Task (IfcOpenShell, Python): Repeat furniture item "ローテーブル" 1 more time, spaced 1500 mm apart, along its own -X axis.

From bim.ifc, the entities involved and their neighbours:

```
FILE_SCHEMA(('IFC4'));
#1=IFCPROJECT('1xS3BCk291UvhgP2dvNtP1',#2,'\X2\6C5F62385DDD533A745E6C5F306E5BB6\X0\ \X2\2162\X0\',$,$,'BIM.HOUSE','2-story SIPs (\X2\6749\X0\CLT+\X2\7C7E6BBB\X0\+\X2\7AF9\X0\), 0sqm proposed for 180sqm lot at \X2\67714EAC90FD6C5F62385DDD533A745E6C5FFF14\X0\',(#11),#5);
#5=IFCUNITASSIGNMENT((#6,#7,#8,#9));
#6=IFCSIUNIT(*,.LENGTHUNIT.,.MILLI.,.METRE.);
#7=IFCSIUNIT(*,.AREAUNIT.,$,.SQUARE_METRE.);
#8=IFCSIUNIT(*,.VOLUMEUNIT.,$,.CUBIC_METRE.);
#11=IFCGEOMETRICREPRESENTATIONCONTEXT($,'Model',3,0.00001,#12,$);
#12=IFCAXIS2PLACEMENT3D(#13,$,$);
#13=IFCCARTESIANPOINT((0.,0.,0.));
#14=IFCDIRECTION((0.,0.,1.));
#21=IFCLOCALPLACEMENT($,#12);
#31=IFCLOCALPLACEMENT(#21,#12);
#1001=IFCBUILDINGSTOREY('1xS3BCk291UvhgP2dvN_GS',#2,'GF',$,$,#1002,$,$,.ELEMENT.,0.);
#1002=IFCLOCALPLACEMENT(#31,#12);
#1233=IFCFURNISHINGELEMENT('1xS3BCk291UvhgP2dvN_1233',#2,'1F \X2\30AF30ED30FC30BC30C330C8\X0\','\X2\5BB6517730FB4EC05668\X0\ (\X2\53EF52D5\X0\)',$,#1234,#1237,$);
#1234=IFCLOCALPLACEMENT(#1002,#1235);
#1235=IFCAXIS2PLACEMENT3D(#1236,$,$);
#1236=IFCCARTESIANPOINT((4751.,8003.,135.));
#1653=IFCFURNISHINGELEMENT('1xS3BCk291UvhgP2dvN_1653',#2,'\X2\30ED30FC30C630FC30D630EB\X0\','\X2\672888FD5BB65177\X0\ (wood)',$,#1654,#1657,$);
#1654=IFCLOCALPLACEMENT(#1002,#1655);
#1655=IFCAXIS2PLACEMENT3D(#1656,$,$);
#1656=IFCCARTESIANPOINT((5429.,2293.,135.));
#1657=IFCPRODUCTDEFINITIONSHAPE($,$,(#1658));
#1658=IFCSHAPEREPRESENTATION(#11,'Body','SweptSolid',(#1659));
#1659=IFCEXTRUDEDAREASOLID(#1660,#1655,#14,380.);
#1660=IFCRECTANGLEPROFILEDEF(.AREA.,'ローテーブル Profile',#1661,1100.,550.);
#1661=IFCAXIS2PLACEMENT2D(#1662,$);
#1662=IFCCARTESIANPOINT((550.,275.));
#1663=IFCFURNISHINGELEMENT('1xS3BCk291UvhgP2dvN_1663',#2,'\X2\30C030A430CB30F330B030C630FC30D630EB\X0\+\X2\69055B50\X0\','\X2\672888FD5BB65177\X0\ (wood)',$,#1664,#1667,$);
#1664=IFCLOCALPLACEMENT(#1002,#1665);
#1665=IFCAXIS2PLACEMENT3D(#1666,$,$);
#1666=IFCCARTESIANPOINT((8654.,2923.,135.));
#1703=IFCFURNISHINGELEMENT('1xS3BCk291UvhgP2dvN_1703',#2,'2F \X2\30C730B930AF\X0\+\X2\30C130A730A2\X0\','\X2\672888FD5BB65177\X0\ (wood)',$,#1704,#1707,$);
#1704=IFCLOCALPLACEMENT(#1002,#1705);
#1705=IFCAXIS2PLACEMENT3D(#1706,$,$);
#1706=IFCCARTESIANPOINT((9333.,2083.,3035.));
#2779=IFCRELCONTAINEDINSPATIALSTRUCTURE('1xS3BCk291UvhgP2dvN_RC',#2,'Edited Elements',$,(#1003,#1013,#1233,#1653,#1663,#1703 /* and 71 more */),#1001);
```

```python
import ifcopenshell
import ifcopenshell.api.geometry
import ifcopenshell.api.root
import ifcopenshell.util.element
import ifcopenshell.util.placement
import ifcopenshell.util.unit

model = ifcopenshell.open("bim.ifc")
unit_scale = ifcopenshell.util.unit.calculate_unit_scale(model)


def reuse_history(source, copy):
    """copy_class also copies each property set's owner history, people and application; keep the originals."""
    for rel in copy.IsDefinedBy:
        if rel.is_a("IfcRelDefinesByProperties") and (history := rel.RelatingPropertyDefinition.OwnerHistory):
            rel.RelatingPropertyDefinition.OwnerHistory = source.OwnerHistory
            ifcopenshell.util.element.remove_deep2(model, history)


source = model.by_guid("1xS3BCk291UvhgP2dvN_1653")
base = ifcopenshell.util.placement.get_local_placement(source.ObjectPlacement)
step = -base[:3, 0] * 1.5 / unit_scale

for i in range(1, 2):
    copy = ifcopenshell.api.root.copy_class(model, product=source)
    copy.Representation = ifcopenshell.util.element.copy_deep(
        model, source.Representation, exclude=["IfcGeometricRepresentationContext", "IfcRepresentationMap"]
    )
    reuse_history(source, copy)
    matrix = base.copy()
    matrix[:3, 3] += i * step
    print("added at", matrix[:3, 3].round(3) + 0.0)
    ifcopenshell.api.geometry.edit_object_placement(model, product=copy, matrix=matrix, is_si=False)

model.write("bim-out.ifc")
```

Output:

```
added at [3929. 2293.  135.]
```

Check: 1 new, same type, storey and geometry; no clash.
